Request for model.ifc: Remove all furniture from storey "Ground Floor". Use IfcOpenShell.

First a look at what the model holds.

```python
import ifcopenshell
import ifcopenshell.util.element

model = ifcopenshell.open("model.ifc")
print(model.schema)
storey = next(s for s in model.by_type("IfcBuildingStorey") if s.Name == "Ground Floor")
furniture = [e for e in ifcopenshell.util.element.get_decomposition(storey) if e.is_a("IfcFurnishingElement")]
seen = {}
for e in furniture:
    element_type = ifcopenshell.util.element.get_type(e)
    name = element_type.Name if element_type not in (None, e) else None
    seen[name] = seen.get(name, 0) + 1
for name, count in sorted(seen.items(), key=str):
    print(count, "x", name)
```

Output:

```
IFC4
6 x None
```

```python
import ifcopenshell
import ifcopenshell.api.root
import ifcopenshell.util.element

model = ifcopenshell.open("model.ifc")

storey = next(s for s in model.by_type("IfcBuildingStorey") if s.Name == "Ground Floor")
furniture = [e for e in ifcopenshell.util.element.get_decomposition(storey) if e.is_a("IfcFurnishingElement")]

for e in furniture:
    ifcopenshell.api.root.remove_product(model, product=e)
print(len(furniture), "removed")

model.write("model_v2.ifc")
```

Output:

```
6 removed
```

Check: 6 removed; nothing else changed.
